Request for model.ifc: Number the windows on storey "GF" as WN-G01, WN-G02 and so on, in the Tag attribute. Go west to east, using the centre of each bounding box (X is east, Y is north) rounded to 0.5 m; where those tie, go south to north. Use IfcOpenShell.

First a look at what the model holds.

```python
import ifcopenshell
import ifcopenshell.util.element
import ifcopenshell.util.placement

model = ifcopenshell.open("model.ifc")
print(model.schema)
storey = next(s for s in model.by_type("IfcBuildingStorey") if s.Name == "GF")
windows = [e for e in ifcopenshell.util.element.get_decomposition(storey) if e.is_a("IfcWindow")]
for e in sorted(windows, key=lambda e: e.id()):
    origin = ifcopenshell.util.placement.get_local_placement(e.ObjectPlacement)[:3, 3]
    print(e.id(), e.Tag, e.Name, origin.round(2) + 0.0, sep=" | ")
```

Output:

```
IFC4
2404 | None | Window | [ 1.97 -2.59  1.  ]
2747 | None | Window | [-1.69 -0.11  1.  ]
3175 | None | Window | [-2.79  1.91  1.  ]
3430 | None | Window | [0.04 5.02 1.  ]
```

```python
import ifcopenshell
import ifcopenshell.geom
import ifcopenshell.util.element
import ifcopenshell.util.shape

model = ifcopenshell.open("model.ifc")
settings = ifcopenshell.geom.settings()
settings.set("use-world-coords", True)


def centre(element):
    shape = ifcopenshell.geom.create_shape(settings, element)
    return ifcopenshell.util.shape.get_bbox_centroid(shape.geometry)


storey = next(s for s in model.by_type("IfcBuildingStorey") if s.Name == "GF")
windows = [e for e in ifcopenshell.util.element.get_decomposition(storey) if e.is_a("IfcWindow")]

# Insertion points can sit at a corner or the storey origin, so sort by the geometry (in metres).
centres = {e: centre(e) for e in windows}
windows.sort(key=lambda e: (round(centres[e][0] / 0.5), centres[e][1]))

for i, e in enumerate(windows, start=1):
    number = f"WN-G{i:02d}"
    e.Tag = number
    print(e.id(), number)

model.write("model_rev.ifc")
```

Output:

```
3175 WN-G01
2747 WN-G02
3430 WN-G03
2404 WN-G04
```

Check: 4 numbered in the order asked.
